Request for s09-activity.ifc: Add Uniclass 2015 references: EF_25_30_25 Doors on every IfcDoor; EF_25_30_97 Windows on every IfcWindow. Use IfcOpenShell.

First a look at what the model holds.

```python
import ifcopenshell

model = ifcopenshell.open("s09-activity.ifc")
print(model.schema)
print("classifications:", [c.Name for c in model.by_type("IfcClassification")])
for ifc_class in ("IfcDoor", "IfcRoof", "IfcStair", "IfcWall", "IfcWindow"):
    print(ifc_class, len(model.by_type(ifc_class)))
```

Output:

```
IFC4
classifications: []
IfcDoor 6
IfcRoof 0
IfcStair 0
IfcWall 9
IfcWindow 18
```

```python
import ifcopenshell
import ifcopenshell.api.classification

model = ifcopenshell.open("s09-activity.ifc")

system = ifcopenshell.api.classification.add_classification(model, classification="Uniclass 2015")

codes = {
    "IfcDoor": ("EF_25_30_25", "Doors"),
    "IfcWindow": ("EF_25_30_97", "Windows"),
}
for ifc_class, (code, name) in codes.items():
    products = model.by_type(ifc_class)
    ifcopenshell.api.classification.add_reference(
        model, products=products, classification=system, identification=code, name=name
    )
    print(code, len(products))

model.write("s09-activity_rev.ifc")
```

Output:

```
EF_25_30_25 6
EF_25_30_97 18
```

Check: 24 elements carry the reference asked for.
